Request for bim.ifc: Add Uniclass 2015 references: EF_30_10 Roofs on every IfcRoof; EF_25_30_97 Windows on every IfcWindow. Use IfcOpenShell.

First a look at what the model holds.

```python
import ifcopenshell

model = ifcopenshell.open("bim.ifc")
print(model.schema)
print("classifications:", [c.Name for c in model.by_type("IfcClassification")])
for ifc_class in ("IfcDoor", "IfcRoof", "IfcStair", "IfcWall", "IfcWindow"):
    print(ifc_class, len(model.by_type(ifc_class)))
```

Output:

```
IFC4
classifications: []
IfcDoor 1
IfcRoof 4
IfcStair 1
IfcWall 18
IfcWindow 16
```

```python
import ifcopenshell
import ifcopenshell.api.classification

model = ifcopenshell.open("bim.ifc")

system = ifcopenshell.api.classification.add_classification(model, classification="Uniclass 2015")

codes = {
    "IfcRoof": ("EF_30_10", "Roofs"),
    "IfcWindow": ("EF_25_30_97", "Windows"),
}
for ifc_class, (code, name) in codes.items():
    products = model.by_type(ifc_class)
    ifcopenshell.api.classification.add_reference(
        model, products=products, classification=system, identification=code, name=name
    )
    print(code, len(products))

model.write("bim_rev.ifc")
```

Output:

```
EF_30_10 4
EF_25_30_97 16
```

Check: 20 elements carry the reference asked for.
